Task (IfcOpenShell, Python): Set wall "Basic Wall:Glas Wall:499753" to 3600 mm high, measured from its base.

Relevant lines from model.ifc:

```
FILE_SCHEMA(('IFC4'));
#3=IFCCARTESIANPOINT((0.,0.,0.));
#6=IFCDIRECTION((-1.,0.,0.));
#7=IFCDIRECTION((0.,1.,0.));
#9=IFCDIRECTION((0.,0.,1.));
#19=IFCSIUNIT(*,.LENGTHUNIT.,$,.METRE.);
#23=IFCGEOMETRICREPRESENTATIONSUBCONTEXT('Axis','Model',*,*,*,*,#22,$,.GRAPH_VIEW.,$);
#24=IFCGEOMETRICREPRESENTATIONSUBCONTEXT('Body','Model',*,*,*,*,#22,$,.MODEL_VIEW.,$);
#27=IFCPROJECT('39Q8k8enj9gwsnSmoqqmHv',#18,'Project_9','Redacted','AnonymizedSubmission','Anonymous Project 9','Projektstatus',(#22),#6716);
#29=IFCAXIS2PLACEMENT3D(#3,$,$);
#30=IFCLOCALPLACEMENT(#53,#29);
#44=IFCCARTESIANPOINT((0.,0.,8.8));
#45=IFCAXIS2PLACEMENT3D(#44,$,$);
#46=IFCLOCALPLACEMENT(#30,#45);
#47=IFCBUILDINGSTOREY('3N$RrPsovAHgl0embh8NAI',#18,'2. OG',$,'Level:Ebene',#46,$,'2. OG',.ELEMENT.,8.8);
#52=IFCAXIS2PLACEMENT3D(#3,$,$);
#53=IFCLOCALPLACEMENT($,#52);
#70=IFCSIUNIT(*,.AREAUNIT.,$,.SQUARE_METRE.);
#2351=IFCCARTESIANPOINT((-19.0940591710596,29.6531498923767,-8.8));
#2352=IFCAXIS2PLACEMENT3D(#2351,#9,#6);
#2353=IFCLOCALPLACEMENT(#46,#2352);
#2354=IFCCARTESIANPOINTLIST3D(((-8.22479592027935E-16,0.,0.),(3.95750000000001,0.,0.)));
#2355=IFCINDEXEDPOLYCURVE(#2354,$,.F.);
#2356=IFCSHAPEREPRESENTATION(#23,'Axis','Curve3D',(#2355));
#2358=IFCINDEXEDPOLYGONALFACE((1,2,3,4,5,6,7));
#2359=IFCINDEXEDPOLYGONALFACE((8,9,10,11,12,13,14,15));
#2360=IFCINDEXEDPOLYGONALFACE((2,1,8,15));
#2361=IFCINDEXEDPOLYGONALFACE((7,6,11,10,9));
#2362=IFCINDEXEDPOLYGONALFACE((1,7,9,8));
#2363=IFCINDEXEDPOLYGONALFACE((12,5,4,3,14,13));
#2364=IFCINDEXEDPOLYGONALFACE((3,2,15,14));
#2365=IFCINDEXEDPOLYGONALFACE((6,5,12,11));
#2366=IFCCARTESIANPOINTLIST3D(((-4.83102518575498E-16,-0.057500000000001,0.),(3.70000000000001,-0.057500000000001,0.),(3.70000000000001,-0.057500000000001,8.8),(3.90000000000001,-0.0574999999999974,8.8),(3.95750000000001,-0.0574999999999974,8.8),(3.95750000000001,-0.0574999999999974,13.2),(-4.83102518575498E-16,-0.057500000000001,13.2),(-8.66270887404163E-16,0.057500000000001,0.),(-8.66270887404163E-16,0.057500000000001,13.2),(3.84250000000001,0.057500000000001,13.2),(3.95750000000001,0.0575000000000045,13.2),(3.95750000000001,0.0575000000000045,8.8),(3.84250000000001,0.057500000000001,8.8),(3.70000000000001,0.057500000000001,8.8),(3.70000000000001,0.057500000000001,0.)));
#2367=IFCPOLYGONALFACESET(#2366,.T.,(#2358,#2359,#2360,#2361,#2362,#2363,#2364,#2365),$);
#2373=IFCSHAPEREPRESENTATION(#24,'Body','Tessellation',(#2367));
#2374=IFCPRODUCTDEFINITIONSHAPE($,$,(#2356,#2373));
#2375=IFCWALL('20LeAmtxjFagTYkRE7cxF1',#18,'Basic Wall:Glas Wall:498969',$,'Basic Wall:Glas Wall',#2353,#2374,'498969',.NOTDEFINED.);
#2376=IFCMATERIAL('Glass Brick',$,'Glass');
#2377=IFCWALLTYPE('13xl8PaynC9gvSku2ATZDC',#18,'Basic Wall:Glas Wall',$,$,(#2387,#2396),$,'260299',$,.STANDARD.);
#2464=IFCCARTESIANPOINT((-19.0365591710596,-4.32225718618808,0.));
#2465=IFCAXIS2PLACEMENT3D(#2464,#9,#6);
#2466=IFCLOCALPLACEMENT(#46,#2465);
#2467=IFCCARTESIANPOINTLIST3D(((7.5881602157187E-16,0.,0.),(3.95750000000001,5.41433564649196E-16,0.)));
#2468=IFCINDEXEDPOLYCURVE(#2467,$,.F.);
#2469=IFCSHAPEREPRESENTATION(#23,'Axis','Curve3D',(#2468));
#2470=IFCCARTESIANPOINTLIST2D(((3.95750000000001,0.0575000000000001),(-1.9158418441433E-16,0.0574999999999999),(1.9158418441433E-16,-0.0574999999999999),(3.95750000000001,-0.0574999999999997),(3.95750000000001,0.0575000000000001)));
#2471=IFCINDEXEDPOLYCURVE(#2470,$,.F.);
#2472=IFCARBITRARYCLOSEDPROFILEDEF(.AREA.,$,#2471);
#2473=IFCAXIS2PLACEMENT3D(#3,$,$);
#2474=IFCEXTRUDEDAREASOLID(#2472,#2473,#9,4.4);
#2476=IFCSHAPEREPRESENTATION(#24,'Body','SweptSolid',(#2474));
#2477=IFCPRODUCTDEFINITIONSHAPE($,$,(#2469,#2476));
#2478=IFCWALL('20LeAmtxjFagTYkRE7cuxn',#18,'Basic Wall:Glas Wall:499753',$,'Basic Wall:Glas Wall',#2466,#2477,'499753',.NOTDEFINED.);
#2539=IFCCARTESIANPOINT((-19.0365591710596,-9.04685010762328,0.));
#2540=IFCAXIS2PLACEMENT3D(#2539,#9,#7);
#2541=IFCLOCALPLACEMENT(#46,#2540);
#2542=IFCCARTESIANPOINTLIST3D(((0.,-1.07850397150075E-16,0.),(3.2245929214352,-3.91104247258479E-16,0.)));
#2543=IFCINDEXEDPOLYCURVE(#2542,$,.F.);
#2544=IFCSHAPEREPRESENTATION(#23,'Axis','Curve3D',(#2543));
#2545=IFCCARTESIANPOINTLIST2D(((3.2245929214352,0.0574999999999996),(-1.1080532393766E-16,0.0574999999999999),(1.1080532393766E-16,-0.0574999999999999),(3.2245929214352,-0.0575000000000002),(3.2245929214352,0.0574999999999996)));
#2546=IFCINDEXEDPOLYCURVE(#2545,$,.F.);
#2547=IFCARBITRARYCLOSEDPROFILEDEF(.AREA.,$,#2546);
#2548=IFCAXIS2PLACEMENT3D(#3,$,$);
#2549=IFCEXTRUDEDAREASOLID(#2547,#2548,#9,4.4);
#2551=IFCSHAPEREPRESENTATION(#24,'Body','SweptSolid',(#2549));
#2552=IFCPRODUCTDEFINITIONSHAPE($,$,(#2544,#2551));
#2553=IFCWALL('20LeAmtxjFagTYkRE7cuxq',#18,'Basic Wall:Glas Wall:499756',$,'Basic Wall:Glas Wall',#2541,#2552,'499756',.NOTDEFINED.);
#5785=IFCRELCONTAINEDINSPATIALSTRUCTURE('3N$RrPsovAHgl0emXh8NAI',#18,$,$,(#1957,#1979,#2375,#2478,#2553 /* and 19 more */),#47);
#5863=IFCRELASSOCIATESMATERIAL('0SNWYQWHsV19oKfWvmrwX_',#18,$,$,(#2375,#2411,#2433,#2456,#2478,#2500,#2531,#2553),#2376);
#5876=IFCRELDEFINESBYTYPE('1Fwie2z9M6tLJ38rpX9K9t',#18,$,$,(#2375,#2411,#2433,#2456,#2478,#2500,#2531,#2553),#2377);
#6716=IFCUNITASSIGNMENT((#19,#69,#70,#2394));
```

```python
import ifcopenshell
import ifcopenshell.geom
import ifcopenshell.util.representation
import ifcopenshell.util.shape
import ifcopenshell.util.unit

model = ifcopenshell.open("model.ifc")
unit_scale = ifcopenshell.util.unit.calculate_unit_scale(model)
settings = ifcopenshell.geom.settings()


def volume(element):
    """Net volume in cubic metres, openings subtracted."""
    shape = ifcopenshell.geom.create_shape(settings, element)
    return ifcopenshell.util.shape.get_volume(shape.geometry)


wall = model.by_guid("20LeAmtxjFagTYkRE7cuxn")
before = volume(wall)

body = ifcopenshell.util.representation.get_representation(wall, "Model", "Body")
solid = body.Items[0]
old_height = solid.Depth
solid.Depth = 3.6 / unit_scale
after = volume(wall)

print(f"height {old_height:g} -> {solid.Depth:g}, volume {before:.3f} -> {after:.3f} m3")

model.write("model_edited.ifc")
```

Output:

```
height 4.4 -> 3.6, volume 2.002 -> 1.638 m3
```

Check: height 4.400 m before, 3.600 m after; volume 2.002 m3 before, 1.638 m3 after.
